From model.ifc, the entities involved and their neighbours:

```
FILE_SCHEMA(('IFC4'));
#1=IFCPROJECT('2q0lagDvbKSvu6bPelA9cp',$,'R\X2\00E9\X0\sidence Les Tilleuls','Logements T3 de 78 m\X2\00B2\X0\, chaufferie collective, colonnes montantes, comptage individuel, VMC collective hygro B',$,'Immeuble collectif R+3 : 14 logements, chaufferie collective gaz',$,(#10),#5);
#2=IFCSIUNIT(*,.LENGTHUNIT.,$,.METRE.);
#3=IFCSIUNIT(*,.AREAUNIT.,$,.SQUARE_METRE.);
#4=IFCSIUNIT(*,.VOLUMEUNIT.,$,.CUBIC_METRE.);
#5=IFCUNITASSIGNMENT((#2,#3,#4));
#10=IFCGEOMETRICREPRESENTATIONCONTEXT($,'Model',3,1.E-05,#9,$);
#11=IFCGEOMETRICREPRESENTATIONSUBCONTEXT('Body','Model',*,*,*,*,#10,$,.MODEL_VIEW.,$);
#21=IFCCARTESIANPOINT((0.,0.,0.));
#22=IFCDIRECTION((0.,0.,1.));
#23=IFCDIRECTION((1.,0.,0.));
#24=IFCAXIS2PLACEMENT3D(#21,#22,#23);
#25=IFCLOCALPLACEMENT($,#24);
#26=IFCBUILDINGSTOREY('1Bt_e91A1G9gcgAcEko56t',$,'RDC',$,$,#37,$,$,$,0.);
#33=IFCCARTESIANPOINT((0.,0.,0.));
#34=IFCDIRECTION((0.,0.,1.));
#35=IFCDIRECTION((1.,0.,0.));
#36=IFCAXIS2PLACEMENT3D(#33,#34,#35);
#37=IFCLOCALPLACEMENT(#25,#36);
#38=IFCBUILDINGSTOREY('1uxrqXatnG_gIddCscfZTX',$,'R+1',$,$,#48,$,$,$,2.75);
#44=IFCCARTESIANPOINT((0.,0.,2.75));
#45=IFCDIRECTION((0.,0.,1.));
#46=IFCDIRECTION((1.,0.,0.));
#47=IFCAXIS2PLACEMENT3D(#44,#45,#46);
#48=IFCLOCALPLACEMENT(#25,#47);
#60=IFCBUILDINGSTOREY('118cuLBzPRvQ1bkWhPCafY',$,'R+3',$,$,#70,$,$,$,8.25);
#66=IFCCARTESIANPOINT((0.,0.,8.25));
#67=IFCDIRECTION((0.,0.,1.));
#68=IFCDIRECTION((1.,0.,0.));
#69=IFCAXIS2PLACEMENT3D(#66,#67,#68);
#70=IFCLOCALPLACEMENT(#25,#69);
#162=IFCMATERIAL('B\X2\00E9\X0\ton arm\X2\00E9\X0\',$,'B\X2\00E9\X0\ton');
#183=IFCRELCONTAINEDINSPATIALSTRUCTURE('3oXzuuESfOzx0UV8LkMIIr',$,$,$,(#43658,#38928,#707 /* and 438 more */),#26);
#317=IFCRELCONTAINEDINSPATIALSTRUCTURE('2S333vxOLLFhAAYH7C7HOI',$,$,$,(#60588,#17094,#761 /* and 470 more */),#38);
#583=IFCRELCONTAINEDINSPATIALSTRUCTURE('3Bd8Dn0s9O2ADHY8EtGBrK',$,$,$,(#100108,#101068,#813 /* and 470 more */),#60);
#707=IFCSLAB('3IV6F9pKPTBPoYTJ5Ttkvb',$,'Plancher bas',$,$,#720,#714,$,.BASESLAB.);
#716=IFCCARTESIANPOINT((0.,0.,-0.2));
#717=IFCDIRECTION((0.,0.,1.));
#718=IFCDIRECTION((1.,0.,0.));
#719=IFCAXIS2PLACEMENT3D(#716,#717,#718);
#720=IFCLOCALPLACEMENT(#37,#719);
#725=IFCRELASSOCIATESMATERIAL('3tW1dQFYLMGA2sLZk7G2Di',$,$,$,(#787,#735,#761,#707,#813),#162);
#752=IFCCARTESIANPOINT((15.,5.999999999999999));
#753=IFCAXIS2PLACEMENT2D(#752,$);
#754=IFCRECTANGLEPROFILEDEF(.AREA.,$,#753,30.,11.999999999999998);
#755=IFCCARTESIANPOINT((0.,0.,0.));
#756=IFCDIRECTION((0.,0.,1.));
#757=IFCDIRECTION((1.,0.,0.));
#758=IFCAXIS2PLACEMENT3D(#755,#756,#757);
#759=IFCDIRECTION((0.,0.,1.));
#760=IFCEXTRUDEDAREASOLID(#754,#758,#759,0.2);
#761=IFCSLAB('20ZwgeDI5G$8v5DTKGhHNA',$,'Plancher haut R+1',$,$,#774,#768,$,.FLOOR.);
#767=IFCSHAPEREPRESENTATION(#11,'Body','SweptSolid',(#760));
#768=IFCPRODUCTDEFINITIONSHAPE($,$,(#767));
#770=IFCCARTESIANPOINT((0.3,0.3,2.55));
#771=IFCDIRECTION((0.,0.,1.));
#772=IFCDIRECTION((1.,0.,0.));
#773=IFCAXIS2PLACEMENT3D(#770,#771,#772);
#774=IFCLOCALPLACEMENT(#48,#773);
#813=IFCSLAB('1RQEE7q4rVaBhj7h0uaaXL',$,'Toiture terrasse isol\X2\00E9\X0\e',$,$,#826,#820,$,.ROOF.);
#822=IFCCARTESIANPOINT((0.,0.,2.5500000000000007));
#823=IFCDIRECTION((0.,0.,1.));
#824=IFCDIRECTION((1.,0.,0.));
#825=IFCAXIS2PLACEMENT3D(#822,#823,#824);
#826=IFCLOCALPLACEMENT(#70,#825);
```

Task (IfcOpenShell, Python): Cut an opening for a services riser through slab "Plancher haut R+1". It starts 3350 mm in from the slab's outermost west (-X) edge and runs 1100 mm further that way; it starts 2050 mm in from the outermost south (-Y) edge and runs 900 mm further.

```python
import numpy as np
import ifcopenshell
import ifcopenshell.api.feature
import ifcopenshell.api.geometry
import ifcopenshell.api.root
import ifcopenshell.geom
import ifcopenshell.util.placement
import ifcopenshell.util.representation
import ifcopenshell.util.shape
import ifcopenshell.util.unit

model = ifcopenshell.open("model.ifc")
unit_scale = ifcopenshell.util.unit.calculate_unit_scale(model)
settings = ifcopenshell.geom.settings()


def volume(element):
    """Net volume in cubic metres, openings subtracted."""
    shape = ifcopenshell.geom.create_shape(settings, element)
    return ifcopenshell.util.shape.get_volume(shape.geometry)


slab = model.by_guid("20ZwgeDI5G$8v5DTKGhHNA")
before = volume(slab)

# Extent in the slab's own axes, in metres. The edges named are its -X and -Y sides.
slab_shape = ifcopenshell.geom.create_shape(settings, slab)
vertices = ifcopenshell.util.shape.get_vertices(slab_shape.geometry)
x_min, y_min, bottom = vertices.min(axis=0)
top = vertices[:, 2].max()

opening = ifcopenshell.api.root.create_entity(model, ifc_class="IfcOpeningElement", name="Services riser opening", predefined_type="OPENING")
context = ifcopenshell.util.representation.get_context(model, "Model", "Body", "MODEL_VIEW")
width, depth = 1.1, 0.9
outline = [(0.0, 0.0), (width, 0.0), (width, depth), (0.0, depth), (0.0, 0.0)]
# Overshoot both faces by 50 mm so the cut is clean.
shape = ifcopenshell.api.geometry.add_slab_representation(
    model, context=context, depth=top - bottom + 0.1, polyline=outline
)
ifcopenshell.api.geometry.assign_representation(model, product=opening, representation=shape)

matrix = ifcopenshell.util.placement.get_local_placement(slab.ObjectPlacement)
matrix[:, 3] = matrix @ np.append(np.array([x_min + 3.35, y_min + 2.05, bottom - 0.05]) / unit_scale, 1.0)
ifcopenshell.api.geometry.edit_object_placement(model, product=opening, matrix=matrix, is_si=False)
ifcopenshell.api.feature.add_feature(model, feature=opening, element=slab)

after = volume(slab)

print(f"slab volume {before:.3f} -> {after:.3f} m3")

model.write("model_v2.ifc")
```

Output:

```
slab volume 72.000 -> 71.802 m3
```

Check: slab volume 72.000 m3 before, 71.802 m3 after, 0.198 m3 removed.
